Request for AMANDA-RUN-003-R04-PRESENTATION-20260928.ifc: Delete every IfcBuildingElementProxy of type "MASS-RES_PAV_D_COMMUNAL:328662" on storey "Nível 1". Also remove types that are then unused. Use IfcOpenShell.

First a look at what the model holds.

```python
import ifcopenshell
import ifcopenshell.util.element

model = ifcopenshell.open("AMANDA-RUN-003-R04-PRESENTATION-20260928.ifc")
print(model.schema)
storey = next(s for s in model.by_type("IfcBuildingStorey") if s.Name == "Nível 1")
proxies = [e for e in ifcopenshell.util.element.get_decomposition(storey) if e.is_a("IfcBuildingElementProxy")]
seen = {}
for e in proxies:
    element_type = ifcopenshell.util.element.get_type(e)
    name = element_type.Name if element_type not in (None, e) else None
    seen[name] = seen.get(name, 0) + 1
for name, count in sorted(seen.items(), key=str):
    print(count, "x", name)
```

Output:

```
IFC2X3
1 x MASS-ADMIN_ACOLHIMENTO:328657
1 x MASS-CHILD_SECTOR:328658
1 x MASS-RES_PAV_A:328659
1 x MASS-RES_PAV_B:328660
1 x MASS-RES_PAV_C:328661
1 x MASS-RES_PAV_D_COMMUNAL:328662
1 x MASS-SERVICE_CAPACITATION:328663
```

```python
import ifcopenshell
import ifcopenshell.api.root
import ifcopenshell.util.element

model = ifcopenshell.open("AMANDA-RUN-003-R04-PRESENTATION-20260928.ifc")

storey = next(s for s in model.by_type("IfcBuildingStorey") if s.Name == "Nível 1")
proxies = [e for e in ifcopenshell.util.element.get_decomposition(storey) if e.is_a("IfcBuildingElementProxy")]
targets = [e for e in proxies if (t := ifcopenshell.util.element.get_type(e)) not in (None, e) and t.Name == "MASS-RES_PAV_D_COMMUNAL:328662"]
types = {ifcopenshell.util.element.get_type(e) for e in targets} - {None, *targets}

for e in targets:
    ifcopenshell.api.root.remove_product(model, product=e)
print(len(targets), "removed")

unused = [t for t in types if not ifcopenshell.util.element.get_types(t)]
for t in unused:
    ifcopenshell.api.root.remove_product(model, product=t)
print(len(unused), "unused types removed")

model.write("AMANDA-RUN-003-R04-PRESENTATION-20260928_v2.ifc")
```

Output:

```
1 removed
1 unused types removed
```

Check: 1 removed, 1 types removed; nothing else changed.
